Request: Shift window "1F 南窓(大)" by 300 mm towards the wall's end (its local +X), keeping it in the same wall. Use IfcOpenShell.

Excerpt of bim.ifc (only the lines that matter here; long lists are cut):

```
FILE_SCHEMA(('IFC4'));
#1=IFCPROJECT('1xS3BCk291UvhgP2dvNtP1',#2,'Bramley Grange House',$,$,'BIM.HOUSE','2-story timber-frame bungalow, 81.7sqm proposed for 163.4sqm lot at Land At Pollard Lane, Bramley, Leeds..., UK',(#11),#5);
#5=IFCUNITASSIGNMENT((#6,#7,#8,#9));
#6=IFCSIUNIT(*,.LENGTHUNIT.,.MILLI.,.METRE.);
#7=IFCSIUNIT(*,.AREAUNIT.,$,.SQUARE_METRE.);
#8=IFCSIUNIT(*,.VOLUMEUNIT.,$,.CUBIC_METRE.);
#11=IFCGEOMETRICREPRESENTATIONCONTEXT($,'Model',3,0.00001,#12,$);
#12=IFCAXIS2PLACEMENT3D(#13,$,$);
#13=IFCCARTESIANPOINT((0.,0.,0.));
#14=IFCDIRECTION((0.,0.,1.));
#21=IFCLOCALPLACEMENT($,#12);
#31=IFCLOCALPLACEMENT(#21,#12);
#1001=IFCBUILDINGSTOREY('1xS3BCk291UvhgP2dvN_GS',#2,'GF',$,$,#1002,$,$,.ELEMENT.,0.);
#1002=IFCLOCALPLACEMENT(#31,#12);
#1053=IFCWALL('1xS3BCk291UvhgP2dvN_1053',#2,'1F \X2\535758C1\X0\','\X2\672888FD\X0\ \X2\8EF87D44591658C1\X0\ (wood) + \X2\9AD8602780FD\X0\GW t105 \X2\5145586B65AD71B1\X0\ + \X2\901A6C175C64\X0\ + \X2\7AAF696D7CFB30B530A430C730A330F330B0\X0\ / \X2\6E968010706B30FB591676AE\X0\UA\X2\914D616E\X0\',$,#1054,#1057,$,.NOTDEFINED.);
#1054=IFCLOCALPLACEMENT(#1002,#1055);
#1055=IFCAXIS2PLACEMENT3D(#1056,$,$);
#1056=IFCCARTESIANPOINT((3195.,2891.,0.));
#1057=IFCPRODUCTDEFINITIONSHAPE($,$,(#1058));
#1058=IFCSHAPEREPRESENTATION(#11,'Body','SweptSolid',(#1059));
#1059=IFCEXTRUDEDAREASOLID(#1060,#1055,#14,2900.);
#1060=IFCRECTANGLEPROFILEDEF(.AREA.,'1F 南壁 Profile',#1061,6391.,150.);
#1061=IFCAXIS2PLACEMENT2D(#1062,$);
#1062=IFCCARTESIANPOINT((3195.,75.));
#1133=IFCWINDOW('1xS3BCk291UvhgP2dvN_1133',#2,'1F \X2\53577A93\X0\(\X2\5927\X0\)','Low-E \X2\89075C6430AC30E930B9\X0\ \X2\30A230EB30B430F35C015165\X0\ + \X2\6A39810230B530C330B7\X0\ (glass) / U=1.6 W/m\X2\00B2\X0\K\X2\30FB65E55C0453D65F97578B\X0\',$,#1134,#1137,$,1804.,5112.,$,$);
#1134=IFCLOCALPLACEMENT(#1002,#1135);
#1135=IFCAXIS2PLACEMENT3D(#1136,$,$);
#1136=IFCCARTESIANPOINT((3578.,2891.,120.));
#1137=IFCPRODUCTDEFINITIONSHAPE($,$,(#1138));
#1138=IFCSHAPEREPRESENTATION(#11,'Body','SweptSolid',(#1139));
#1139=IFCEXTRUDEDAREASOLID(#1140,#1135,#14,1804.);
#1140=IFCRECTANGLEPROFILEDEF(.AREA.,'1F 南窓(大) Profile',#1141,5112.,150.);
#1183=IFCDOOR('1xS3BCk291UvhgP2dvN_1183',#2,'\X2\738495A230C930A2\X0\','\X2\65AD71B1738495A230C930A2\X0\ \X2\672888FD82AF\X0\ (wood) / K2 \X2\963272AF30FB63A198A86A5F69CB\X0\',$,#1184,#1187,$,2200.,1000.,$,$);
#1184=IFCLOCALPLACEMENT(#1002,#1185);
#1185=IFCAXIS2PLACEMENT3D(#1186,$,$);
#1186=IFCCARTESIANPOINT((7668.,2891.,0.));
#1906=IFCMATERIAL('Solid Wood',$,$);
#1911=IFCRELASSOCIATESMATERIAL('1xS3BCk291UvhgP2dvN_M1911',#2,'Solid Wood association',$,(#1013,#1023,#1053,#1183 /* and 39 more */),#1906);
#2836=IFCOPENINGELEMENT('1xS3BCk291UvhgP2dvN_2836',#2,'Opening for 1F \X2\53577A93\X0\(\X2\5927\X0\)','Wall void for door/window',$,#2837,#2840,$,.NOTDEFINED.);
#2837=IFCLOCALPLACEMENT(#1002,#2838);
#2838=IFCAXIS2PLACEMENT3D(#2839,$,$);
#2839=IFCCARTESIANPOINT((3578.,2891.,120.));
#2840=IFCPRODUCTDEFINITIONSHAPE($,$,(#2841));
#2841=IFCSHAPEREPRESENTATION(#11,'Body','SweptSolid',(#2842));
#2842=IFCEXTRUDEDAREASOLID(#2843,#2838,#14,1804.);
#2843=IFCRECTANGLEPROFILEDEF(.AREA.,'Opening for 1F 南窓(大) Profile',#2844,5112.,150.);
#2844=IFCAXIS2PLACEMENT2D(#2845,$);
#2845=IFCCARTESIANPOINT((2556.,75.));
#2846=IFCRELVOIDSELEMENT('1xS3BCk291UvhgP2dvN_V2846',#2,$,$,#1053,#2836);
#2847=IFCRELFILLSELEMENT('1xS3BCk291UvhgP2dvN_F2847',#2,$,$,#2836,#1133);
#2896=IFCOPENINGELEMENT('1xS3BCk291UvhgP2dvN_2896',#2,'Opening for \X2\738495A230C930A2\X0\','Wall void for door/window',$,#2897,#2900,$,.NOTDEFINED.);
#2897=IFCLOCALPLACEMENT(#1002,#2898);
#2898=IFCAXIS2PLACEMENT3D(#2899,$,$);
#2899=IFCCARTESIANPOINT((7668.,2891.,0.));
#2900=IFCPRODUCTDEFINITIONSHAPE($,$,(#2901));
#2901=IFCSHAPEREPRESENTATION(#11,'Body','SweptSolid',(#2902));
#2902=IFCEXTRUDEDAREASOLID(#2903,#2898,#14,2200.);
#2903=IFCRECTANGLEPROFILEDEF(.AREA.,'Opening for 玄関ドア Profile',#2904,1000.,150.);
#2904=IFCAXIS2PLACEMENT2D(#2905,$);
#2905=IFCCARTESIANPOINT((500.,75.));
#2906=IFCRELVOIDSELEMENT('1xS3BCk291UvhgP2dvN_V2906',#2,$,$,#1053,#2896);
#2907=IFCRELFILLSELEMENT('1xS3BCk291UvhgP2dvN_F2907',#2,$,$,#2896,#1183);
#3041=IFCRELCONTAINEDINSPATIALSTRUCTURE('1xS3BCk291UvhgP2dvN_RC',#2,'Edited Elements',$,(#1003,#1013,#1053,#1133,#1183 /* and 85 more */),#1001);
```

```python
import ifcopenshell
import ifcopenshell.api.geometry
import ifcopenshell.util.placement
import ifcopenshell.util.unit

model = ifcopenshell.open("bim.ifc")
unit_scale = ifcopenshell.util.unit.calculate_unit_scale(model)

window = model.by_guid("1xS3BCk291UvhgP2dvN_1133")
opening = window.FillsVoids[0].RelatingOpeningElement
wall = opening.VoidsElements[0].RelatingBuildingElement

wall_matrix = ifcopenshell.util.placement.get_local_placement(wall.ObjectPlacement)
shift = wall_matrix[:3, 0] * 0.3 / unit_scale
before = ifcopenshell.util.placement.get_local_placement(window.ObjectPlacement)[:3, 3].copy()

# The window is not placed relative to its opening, so move both.
for product in (opening, window):
    matrix = ifcopenshell.util.placement.get_local_placement(product.ObjectPlacement)
    matrix[:3, 3] += shift
    ifcopenshell.api.geometry.edit_object_placement(model, product=product, matrix=matrix, is_si=False)

after = ifcopenshell.util.placement.get_local_placement(window.ObjectPlacement)[:3, 3]
print("window moved by", (after - before).round(3) + 0.0)

model.write("bim_edited.ifc")
```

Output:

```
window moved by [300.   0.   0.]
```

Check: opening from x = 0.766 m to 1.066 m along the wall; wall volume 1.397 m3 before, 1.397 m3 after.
